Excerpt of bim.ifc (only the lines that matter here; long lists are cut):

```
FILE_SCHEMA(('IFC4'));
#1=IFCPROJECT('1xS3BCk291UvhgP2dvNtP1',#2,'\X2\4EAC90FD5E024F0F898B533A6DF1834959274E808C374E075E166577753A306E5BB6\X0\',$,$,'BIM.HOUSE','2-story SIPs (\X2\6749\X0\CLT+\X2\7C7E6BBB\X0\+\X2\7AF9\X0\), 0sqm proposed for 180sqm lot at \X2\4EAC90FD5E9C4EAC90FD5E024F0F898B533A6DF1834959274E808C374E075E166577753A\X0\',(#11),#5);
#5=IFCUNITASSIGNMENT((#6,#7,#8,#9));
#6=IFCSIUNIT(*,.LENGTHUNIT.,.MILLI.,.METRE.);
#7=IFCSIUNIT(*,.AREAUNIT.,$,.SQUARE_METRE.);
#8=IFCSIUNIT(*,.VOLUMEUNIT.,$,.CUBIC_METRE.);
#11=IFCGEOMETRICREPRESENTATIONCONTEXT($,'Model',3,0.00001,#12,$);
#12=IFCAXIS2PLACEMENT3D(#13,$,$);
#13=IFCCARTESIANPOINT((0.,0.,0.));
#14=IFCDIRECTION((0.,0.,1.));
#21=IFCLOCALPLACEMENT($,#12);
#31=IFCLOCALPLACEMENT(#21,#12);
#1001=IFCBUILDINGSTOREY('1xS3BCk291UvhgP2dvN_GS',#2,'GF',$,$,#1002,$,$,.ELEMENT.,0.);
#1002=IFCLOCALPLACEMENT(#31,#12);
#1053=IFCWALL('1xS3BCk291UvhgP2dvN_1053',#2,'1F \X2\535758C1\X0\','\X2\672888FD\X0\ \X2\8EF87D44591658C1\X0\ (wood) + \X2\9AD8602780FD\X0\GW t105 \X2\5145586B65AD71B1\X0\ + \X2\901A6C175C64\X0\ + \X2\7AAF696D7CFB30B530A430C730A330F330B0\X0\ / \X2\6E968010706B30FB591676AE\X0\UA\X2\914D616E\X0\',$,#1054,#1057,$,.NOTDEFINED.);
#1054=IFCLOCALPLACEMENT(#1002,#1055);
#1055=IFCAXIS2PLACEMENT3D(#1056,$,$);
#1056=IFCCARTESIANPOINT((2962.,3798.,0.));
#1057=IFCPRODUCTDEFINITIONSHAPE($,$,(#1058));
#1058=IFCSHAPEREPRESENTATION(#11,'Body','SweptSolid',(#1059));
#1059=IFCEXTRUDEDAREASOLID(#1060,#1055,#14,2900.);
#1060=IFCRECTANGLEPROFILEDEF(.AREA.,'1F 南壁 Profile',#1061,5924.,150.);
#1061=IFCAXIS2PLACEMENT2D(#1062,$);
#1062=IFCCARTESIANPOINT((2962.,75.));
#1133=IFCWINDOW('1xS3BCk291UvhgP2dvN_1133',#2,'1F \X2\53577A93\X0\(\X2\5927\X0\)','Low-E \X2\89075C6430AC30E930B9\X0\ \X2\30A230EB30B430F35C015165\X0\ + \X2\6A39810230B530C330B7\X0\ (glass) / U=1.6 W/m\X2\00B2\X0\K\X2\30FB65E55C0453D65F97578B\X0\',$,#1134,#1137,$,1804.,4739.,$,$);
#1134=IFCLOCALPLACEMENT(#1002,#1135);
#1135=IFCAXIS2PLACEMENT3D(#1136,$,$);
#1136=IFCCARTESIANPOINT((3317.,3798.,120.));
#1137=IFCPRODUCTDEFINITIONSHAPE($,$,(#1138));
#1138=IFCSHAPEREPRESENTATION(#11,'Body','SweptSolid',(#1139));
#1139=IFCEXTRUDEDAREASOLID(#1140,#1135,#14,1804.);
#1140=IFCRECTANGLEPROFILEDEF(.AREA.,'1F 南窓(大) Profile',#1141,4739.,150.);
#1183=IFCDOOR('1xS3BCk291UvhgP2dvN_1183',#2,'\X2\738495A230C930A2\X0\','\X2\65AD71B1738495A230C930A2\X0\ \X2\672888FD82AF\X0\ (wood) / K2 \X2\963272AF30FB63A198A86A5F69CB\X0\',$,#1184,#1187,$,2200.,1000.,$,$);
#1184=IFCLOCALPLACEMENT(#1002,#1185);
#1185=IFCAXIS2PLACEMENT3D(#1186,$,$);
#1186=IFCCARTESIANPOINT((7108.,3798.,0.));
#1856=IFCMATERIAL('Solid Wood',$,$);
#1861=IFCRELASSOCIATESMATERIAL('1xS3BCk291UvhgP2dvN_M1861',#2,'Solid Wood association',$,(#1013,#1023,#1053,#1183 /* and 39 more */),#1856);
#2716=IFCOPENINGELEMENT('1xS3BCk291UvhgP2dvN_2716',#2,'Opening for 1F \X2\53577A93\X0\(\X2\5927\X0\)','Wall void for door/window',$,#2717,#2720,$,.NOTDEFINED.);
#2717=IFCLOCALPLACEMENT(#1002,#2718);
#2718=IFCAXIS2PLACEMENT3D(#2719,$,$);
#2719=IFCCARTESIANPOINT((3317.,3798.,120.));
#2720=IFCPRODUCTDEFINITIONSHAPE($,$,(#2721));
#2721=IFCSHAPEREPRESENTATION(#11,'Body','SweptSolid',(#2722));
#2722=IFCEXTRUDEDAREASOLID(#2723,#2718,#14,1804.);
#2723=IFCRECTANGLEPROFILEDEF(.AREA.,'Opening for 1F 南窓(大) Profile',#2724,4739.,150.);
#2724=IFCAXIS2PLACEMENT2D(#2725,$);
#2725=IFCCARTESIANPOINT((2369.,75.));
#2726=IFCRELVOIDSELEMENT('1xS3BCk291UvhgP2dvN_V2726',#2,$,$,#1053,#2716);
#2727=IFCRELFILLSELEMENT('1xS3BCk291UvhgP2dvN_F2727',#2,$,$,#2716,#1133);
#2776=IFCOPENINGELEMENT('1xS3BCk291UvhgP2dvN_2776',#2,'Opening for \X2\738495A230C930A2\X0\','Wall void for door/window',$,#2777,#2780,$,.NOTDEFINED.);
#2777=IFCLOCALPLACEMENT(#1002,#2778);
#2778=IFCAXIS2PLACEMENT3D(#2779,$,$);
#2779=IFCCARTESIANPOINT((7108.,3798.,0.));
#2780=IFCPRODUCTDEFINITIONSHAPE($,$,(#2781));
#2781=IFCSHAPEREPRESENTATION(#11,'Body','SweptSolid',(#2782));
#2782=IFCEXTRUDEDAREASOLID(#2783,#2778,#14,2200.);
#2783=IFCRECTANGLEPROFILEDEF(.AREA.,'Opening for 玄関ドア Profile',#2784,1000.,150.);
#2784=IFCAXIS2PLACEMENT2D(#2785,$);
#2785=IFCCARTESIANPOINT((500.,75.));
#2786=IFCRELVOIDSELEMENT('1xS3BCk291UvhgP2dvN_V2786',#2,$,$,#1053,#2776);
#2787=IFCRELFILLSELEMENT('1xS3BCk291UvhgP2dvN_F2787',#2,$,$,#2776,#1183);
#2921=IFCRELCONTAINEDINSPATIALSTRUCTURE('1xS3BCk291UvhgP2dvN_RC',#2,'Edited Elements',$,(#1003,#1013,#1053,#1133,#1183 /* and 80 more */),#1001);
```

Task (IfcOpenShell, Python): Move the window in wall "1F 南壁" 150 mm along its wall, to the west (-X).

```python
import ifcopenshell
import ifcopenshell.api.geometry
import ifcopenshell.util.placement

model = ifcopenshell.open("bim.ifc")

window = model.by_guid("1xS3BCk291UvhgP2dvN_1133")
opening = window.FillsVoids[0].RelatingOpeningElement
wall = opening.VoidsElements[0].RelatingBuildingElement

wall_matrix = ifcopenshell.util.placement.get_local_placement(wall.ObjectPlacement)
shift = wall_matrix[:3, 0] * -150.0
before = ifcopenshell.util.placement.get_local_placement(window.ObjectPlacement)[:3, 3].copy()

# The window is not placed relative to its opening, so move both.
for product in (opening, window):
    matrix = ifcopenshell.util.placement.get_local_placement(product.ObjectPlacement)
    matrix[:3, 3] += shift
    ifcopenshell.api.geometry.edit_object_placement(model, product=product, matrix=matrix, is_si=False)

after = ifcopenshell.util.placement.get_local_placement(window.ObjectPlacement)[:3, 3]
print("window moved by", (after - before).round(3) + 0.0)

model.write("bim_rev.ifc")
```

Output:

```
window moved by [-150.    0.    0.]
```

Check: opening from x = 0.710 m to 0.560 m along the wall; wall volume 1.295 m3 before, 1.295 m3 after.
